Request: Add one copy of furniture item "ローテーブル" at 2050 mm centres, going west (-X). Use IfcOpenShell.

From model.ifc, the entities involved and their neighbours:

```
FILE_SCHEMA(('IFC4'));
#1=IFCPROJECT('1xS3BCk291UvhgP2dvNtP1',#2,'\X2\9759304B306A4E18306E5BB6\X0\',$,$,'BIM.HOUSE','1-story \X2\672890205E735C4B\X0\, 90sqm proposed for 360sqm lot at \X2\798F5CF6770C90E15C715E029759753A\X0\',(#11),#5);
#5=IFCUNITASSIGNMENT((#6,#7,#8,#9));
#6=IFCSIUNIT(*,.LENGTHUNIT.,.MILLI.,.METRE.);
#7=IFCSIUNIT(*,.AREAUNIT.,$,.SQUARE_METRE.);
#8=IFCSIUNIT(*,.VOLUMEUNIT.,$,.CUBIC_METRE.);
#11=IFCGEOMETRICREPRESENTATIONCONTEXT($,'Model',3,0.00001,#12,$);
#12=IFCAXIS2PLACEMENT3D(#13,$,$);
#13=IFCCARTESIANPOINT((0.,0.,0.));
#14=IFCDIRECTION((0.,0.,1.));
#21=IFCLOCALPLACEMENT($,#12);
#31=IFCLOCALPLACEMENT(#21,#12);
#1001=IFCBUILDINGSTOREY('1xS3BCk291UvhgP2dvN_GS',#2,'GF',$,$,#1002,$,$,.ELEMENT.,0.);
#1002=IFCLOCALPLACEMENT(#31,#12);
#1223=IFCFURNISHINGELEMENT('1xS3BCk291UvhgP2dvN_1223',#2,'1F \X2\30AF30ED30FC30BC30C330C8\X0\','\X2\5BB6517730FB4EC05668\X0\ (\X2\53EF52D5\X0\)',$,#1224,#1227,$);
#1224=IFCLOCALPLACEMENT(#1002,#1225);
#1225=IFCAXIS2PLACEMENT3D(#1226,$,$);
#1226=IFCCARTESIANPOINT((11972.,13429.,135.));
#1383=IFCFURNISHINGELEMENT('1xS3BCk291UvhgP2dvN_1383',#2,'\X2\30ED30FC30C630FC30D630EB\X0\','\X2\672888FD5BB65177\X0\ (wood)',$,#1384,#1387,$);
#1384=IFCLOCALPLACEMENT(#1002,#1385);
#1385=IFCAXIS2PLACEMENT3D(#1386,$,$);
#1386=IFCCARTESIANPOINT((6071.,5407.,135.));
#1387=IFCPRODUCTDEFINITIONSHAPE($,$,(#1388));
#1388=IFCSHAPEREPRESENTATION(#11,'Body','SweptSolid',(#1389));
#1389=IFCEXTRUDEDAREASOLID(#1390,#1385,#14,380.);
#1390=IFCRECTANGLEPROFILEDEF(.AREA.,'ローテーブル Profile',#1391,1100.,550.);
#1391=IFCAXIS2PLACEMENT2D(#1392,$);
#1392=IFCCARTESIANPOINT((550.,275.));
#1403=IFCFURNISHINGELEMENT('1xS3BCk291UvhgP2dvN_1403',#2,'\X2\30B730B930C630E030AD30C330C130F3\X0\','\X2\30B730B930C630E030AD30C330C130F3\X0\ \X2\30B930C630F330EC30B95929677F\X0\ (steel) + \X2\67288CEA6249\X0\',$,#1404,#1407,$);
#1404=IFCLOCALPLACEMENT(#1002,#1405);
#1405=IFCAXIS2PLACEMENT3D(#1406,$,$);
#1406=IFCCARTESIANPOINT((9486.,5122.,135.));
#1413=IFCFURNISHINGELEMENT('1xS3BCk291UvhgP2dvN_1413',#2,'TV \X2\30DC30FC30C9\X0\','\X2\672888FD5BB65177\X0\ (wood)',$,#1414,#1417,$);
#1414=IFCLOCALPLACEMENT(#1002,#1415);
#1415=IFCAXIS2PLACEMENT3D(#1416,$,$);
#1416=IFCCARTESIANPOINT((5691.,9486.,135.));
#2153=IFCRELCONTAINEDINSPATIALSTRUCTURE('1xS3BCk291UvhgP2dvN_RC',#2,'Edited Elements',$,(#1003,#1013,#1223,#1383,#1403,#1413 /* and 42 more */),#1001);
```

```python
import numpy as np
import ifcopenshell
import ifcopenshell.api.geometry
import ifcopenshell.api.root
import ifcopenshell.util.element
import ifcopenshell.util.placement
import ifcopenshell.util.unit

model = ifcopenshell.open("model.ifc")
unit_scale = ifcopenshell.util.unit.calculate_unit_scale(model)


def reuse_history(source, copy):
    """copy_class also copies each property set's owner history, people and application; keep the originals."""
    for rel in copy.IsDefinedBy:
        if rel.is_a("IfcRelDefinesByProperties") and (history := rel.RelatingPropertyDefinition.OwnerHistory):
            rel.RelatingPropertyDefinition.OwnerHistory = source.OwnerHistory
            ifcopenshell.util.element.remove_deep2(model, history)


source = model.by_guid("1xS3BCk291UvhgP2dvN_1383")
base = ifcopenshell.util.placement.get_local_placement(source.ObjectPlacement)
step = np.array([-1.0, 0.0, 0.0]) * 2.05 / unit_scale

for i in range(1, 2):
    copy = ifcopenshell.api.root.copy_class(model, product=source)
    copy.Representation = ifcopenshell.util.element.copy_deep(
        model, source.Representation, exclude=["IfcGeometricRepresentationContext", "IfcRepresentationMap"]
    )
    reuse_history(source, copy)
    matrix = base.copy()
    matrix[:3, 3] += i * step
    print("added at", matrix[:3, 3].round(3) + 0.0)
    ifcopenshell.api.geometry.edit_object_placement(model, product=copy, matrix=matrix, is_si=False)

model.write("model_updated.ifc")
```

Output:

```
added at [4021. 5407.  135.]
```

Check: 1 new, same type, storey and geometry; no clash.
